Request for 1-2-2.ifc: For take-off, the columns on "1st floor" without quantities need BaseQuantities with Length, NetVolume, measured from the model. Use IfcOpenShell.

First a look at what the model holds.

```python
import ifcopenshell
import ifcopenshell.util.element
import ifcopenshell.util.unit

model = ifcopenshell.open("1-2-2.ifc")
print(model.schema)
for unit_type in ("LENGTHUNIT", "AREAUNIT", "VOLUMEUNIT"):
    print(unit_type, ifcopenshell.util.unit.calculate_unit_scale(model, unit_type))
storey = next(s for s in model.by_type("IfcBuildingStorey") if s.Name == "1st floor")
columns = [e for e in ifcopenshell.util.element.get_decomposition(storey) if e.is_a("IfcColumn")]
for e in sorted(columns, key=lambda e: e.id()):
    print(e.id(), e.is_a(), e.Name, list(ifcopenshell.util.element.get_psets(e, qtos_only=True)), sep=" | ")
```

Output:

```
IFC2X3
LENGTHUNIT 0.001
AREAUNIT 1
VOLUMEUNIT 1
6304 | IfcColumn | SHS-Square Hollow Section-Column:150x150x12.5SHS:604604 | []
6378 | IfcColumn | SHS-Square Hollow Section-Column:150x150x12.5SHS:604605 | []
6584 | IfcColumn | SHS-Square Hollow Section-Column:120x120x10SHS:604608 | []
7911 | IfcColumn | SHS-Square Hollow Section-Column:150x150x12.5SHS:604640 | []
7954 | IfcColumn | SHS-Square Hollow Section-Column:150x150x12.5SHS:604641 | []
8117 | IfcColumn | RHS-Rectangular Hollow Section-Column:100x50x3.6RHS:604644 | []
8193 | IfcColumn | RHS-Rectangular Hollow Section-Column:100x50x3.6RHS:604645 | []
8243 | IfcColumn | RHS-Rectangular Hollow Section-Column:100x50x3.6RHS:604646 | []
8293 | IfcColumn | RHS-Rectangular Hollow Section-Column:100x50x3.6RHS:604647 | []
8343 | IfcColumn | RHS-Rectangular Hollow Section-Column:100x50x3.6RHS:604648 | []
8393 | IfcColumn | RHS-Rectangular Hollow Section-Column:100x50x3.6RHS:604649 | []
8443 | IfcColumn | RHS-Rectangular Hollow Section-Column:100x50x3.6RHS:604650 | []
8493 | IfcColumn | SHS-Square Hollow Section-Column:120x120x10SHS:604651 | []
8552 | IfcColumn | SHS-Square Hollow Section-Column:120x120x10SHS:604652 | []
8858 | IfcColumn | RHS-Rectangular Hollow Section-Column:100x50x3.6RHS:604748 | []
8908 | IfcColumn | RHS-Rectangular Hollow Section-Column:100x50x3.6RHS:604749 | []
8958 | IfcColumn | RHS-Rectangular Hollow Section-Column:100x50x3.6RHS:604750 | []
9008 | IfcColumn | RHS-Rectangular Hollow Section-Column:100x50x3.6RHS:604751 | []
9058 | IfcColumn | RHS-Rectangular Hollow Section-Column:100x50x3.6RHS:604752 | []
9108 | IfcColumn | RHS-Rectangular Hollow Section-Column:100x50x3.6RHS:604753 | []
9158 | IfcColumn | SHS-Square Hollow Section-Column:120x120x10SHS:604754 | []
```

```python
import ifcopenshell
import ifcopenshell.api.pset
import ifcopenshell.geom
import ifcopenshell.util.element
import ifcopenshell.util.shape
import ifcopenshell.util.unit

model = ifcopenshell.open("1-2-2.ifc")
unit_scale = ifcopenshell.util.unit.calculate_unit_scale(model)
volume_scale = ifcopenshell.util.unit.calculate_unit_scale(model, "VOLUMEUNIT")
settings = ifcopenshell.geom.settings()

storey = next(s for s in model.by_type("IfcBuildingStorey") if s.Name == "1st floor")
columns = [e for e in ifcopenshell.util.element.get_decomposition(storey) if e.is_a("IfcColumn")]

for e in sorted(columns, key=lambda e: e.id()):
    if ifcopenshell.util.element.get_psets(e, qtos_only=True, should_inherit=False):
        continue
    # Geometry comes back in metres, in the element's own axes.
    shape = ifcopenshell.geom.create_shape(settings, e)
    values = {
        "Length": ifcopenshell.util.shape.get_z(shape.geometry) / unit_scale,
        "NetVolume": ifcopenshell.util.shape.get_volume(shape.geometry) / volume_scale,
    }
    qto = ifcopenshell.api.pset.add_qto(model, product=e, name="BaseQuantities")
    ifcopenshell.api.pset.edit_qto(model, qto=qto, properties=values)
    print(e.id(), {k: round(v, 3) for k, v in values.items()})

model.write("1-2-2_updated.ifc")
```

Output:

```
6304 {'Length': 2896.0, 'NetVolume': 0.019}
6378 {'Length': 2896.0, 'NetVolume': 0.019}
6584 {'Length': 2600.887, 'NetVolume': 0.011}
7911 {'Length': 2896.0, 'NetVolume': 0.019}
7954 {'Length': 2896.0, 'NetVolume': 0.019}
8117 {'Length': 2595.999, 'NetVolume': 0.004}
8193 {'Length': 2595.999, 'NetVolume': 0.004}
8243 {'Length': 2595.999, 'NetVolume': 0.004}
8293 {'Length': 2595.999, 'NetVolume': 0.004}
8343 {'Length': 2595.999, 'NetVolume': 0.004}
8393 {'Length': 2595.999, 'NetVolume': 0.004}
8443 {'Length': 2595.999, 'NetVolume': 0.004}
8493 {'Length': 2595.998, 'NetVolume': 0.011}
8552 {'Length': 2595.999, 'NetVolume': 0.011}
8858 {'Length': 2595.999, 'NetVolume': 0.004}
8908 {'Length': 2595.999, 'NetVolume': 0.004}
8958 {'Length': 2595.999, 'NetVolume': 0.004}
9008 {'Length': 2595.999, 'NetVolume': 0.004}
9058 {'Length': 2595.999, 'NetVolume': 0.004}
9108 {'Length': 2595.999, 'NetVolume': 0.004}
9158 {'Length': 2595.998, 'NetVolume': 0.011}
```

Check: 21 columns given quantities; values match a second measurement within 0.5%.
